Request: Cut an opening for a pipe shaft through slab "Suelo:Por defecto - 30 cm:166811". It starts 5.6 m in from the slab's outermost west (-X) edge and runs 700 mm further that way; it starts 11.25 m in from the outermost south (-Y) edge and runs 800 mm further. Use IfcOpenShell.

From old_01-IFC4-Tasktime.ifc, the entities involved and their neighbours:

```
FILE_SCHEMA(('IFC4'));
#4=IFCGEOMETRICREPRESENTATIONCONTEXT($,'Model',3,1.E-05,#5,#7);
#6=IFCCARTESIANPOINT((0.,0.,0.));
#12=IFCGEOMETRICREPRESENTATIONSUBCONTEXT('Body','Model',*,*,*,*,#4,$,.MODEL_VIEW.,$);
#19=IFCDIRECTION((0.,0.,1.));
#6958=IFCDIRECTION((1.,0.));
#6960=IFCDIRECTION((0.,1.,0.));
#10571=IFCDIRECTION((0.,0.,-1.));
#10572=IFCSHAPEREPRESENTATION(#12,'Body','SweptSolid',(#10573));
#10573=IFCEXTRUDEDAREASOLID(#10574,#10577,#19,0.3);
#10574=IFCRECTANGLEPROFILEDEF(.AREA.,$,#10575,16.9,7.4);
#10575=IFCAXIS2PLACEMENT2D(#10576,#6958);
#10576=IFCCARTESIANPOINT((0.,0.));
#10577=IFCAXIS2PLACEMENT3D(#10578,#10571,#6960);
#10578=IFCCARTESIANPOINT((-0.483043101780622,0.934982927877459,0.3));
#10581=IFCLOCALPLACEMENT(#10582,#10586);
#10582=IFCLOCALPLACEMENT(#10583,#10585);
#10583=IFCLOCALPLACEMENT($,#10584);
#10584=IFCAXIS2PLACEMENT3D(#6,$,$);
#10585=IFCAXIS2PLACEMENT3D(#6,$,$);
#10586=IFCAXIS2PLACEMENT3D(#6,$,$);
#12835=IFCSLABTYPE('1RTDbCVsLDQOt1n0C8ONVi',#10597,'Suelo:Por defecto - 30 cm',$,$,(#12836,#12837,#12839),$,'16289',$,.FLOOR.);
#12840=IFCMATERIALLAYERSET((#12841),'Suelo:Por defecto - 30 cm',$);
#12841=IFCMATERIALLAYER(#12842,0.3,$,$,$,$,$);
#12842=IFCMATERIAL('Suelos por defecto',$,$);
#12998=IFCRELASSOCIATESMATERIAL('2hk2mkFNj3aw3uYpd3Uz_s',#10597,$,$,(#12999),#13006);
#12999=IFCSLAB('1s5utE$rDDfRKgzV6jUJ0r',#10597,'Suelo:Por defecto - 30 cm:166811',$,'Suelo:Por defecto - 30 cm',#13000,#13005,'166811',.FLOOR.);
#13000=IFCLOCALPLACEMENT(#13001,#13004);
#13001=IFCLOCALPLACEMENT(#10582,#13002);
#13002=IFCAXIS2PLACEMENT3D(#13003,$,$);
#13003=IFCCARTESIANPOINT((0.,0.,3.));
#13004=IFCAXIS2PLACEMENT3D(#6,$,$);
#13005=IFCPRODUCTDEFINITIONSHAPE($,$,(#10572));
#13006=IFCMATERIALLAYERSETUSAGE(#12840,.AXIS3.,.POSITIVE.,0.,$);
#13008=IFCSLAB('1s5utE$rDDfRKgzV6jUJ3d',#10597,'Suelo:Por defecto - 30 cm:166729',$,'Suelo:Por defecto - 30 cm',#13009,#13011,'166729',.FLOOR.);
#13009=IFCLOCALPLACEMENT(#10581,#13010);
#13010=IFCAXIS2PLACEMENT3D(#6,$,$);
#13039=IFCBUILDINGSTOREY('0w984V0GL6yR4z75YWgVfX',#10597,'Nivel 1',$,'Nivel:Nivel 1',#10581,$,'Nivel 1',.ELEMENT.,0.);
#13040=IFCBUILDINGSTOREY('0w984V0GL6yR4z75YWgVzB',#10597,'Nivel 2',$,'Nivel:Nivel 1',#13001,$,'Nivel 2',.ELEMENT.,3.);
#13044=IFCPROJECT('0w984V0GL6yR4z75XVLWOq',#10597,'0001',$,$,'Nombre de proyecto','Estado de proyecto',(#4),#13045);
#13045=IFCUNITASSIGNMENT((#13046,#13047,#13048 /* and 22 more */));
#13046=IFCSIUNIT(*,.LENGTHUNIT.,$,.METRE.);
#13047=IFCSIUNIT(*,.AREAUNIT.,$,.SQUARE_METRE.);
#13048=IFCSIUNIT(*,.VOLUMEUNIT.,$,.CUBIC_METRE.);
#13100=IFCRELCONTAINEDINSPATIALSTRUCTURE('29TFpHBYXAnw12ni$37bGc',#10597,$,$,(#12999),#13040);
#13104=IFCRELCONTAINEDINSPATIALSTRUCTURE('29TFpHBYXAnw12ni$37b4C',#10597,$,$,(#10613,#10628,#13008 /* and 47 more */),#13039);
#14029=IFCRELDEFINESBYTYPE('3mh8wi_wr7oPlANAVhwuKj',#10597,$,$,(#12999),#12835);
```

```python
import numpy as np
import ifcopenshell
import ifcopenshell.api.feature
import ifcopenshell.api.geometry
import ifcopenshell.api.root
import ifcopenshell.geom
import ifcopenshell.util.placement
import ifcopenshell.util.representation
import ifcopenshell.util.shape
import ifcopenshell.util.unit

model = ifcopenshell.open("old_01-IFC4-Tasktime.ifc")
unit_scale = ifcopenshell.util.unit.calculate_unit_scale(model)
settings = ifcopenshell.geom.settings()


def volume(element):
    """Net volume in cubic metres, openings subtracted."""
    shape = ifcopenshell.geom.create_shape(settings, element)
    return ifcopenshell.util.shape.get_volume(shape.geometry)


slab = model.by_guid("1s5utE$rDDfRKgzV6jUJ0r")
before = volume(slab)

# Extent in the slab's own axes, in metres. The edges named are its -X and -Y sides.
slab_shape = ifcopenshell.geom.create_shape(settings, slab)
vertices = ifcopenshell.util.shape.get_vertices(slab_shape.geometry)
x_min, y_min, bottom = vertices.min(axis=0)
top = vertices[:, 2].max()

opening = ifcopenshell.api.root.create_entity(model, ifc_class="IfcOpeningElement", name="Pipe shaft opening", predefined_type="OPENING")
context = ifcopenshell.util.representation.get_context(model, "Model", "Body", "MODEL_VIEW")
width, depth = 0.7, 0.8
outline = [(0.0, 0.0), (width, 0.0), (width, depth), (0.0, depth), (0.0, 0.0)]
# Overshoot both faces by 50 mm so the cut is clean.
shape = ifcopenshell.api.geometry.add_slab_representation(
    model, context=context, depth=top - bottom + 0.1, polyline=outline
)
ifcopenshell.api.geometry.assign_representation(model, product=opening, representation=shape)

matrix = ifcopenshell.util.placement.get_local_placement(slab.ObjectPlacement)
matrix[:, 3] = matrix @ np.append(np.array([x_min + 5.6, y_min + 11.25, bottom - 0.05]) / unit_scale, 1.0)
ifcopenshell.api.geometry.edit_object_placement(model, product=opening, matrix=matrix, is_si=False)
ifcopenshell.api.feature.add_feature(model, feature=opening, element=slab)

after = volume(slab)

print(f"slab volume {before:.3f} -> {after:.3f} m3")

model.write("old_01-IFC4-Tasktime_v2.ifc")
```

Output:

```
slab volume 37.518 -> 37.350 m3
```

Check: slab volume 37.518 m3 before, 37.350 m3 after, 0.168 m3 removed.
